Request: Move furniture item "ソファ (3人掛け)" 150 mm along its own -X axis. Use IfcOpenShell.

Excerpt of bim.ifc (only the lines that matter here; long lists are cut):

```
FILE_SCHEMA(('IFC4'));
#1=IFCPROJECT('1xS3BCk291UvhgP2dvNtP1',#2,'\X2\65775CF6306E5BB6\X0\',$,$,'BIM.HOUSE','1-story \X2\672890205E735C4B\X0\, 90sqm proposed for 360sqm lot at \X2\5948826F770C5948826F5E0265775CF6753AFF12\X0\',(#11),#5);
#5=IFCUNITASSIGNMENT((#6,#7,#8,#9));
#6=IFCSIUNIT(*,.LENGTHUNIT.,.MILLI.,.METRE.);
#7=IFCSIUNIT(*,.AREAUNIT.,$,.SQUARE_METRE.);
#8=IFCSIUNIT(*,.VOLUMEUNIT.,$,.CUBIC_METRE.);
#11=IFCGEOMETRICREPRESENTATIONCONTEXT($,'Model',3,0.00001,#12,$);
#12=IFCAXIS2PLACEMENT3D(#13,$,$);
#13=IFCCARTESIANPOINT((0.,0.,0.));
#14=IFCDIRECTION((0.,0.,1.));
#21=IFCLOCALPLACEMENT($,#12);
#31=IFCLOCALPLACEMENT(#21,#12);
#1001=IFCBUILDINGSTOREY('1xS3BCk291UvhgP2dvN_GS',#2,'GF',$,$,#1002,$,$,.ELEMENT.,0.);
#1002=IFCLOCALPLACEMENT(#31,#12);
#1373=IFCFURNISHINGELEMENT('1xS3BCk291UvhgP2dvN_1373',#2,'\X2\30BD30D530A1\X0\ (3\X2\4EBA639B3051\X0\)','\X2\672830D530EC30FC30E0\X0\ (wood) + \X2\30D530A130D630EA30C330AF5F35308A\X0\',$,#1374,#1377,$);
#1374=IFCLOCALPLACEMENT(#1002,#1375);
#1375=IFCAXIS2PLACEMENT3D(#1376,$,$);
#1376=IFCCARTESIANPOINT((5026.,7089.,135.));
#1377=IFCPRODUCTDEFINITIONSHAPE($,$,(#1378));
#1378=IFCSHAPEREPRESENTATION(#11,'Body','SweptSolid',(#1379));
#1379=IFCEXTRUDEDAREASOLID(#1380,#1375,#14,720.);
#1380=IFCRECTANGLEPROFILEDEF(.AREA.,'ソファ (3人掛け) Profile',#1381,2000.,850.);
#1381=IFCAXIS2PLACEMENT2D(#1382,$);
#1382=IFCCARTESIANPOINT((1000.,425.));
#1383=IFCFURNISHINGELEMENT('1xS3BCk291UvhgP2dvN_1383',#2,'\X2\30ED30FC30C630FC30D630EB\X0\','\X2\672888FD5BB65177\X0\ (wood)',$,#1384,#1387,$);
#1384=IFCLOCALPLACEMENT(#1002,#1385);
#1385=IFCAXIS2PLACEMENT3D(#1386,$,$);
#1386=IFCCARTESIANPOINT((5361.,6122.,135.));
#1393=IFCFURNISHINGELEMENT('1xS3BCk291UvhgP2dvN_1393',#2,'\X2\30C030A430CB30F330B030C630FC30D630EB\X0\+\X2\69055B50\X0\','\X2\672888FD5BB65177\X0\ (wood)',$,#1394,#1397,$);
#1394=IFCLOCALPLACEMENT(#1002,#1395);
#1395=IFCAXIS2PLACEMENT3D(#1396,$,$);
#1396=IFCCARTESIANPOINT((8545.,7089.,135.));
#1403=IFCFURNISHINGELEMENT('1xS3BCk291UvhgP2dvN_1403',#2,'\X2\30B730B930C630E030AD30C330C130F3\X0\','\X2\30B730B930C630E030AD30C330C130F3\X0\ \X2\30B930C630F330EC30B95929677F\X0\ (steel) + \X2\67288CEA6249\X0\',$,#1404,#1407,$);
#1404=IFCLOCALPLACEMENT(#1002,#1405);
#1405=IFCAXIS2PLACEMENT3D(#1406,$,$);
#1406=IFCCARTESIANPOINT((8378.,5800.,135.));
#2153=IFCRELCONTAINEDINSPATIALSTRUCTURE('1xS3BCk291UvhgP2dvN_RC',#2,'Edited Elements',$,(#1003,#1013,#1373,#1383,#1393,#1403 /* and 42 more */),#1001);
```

```python
import ifcopenshell
import ifcopenshell.api.geometry
import ifcopenshell.util.placement
import ifcopenshell.util.unit

model = ifcopenshell.open("bim.ifc")
unit_scale = ifcopenshell.util.unit.calculate_unit_scale(model)

item = model.by_guid("1xS3BCk291UvhgP2dvN_1373")
matrix = ifcopenshell.util.placement.get_local_placement(item.ObjectPlacement)
matrix[:3, 3] -= matrix[:3, 0] * 0.15 / unit_scale
ifcopenshell.api.geometry.edit_object_placement(model, product=item, matrix=matrix, is_si=False)

print(ifcopenshell.util.placement.get_local_placement(item.ObjectPlacement).round(3) + 0.0)

model.write("bim_updated.ifc")
```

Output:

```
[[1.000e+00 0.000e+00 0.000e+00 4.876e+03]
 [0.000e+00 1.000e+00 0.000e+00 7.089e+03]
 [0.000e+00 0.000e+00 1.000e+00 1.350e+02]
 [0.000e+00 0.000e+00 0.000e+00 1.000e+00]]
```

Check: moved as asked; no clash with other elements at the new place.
